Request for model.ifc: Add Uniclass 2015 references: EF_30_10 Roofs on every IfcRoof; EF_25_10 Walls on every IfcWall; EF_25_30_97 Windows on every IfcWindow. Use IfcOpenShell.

First a look at what the model holds.

```python
import ifcopenshell

model = ifcopenshell.open("model.ifc")
print(model.schema)
print("classifications:", [c.Name for c in model.by_type("IfcClassification")])
for ifc_class in ("IfcDoor", "IfcRoof", "IfcStair", "IfcWall", "IfcWindow"):
    print(ifc_class, len(model.by_type(ifc_class)))
```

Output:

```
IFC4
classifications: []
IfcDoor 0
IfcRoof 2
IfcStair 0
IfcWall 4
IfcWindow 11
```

```python
import ifcopenshell
import ifcopenshell.api.classification

model = ifcopenshell.open("model.ifc")

system = ifcopenshell.api.classification.add_classification(model, classification="Uniclass 2015")

codes = {
    "IfcRoof": ("EF_30_10", "Roofs"),
    "IfcWall": ("EF_25_10", "Walls"),
    "IfcWindow": ("EF_25_30_97", "Windows"),
}
for ifc_class, (code, name) in codes.items():
    products = model.by_type(ifc_class)
    ifcopenshell.api.classification.add_reference(
        model, products=products, classification=system, identification=code, name=name
    )
    print(code, len(products))

model.write("model_rev.ifc")
```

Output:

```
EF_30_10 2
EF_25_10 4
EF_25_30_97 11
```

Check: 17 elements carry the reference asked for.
